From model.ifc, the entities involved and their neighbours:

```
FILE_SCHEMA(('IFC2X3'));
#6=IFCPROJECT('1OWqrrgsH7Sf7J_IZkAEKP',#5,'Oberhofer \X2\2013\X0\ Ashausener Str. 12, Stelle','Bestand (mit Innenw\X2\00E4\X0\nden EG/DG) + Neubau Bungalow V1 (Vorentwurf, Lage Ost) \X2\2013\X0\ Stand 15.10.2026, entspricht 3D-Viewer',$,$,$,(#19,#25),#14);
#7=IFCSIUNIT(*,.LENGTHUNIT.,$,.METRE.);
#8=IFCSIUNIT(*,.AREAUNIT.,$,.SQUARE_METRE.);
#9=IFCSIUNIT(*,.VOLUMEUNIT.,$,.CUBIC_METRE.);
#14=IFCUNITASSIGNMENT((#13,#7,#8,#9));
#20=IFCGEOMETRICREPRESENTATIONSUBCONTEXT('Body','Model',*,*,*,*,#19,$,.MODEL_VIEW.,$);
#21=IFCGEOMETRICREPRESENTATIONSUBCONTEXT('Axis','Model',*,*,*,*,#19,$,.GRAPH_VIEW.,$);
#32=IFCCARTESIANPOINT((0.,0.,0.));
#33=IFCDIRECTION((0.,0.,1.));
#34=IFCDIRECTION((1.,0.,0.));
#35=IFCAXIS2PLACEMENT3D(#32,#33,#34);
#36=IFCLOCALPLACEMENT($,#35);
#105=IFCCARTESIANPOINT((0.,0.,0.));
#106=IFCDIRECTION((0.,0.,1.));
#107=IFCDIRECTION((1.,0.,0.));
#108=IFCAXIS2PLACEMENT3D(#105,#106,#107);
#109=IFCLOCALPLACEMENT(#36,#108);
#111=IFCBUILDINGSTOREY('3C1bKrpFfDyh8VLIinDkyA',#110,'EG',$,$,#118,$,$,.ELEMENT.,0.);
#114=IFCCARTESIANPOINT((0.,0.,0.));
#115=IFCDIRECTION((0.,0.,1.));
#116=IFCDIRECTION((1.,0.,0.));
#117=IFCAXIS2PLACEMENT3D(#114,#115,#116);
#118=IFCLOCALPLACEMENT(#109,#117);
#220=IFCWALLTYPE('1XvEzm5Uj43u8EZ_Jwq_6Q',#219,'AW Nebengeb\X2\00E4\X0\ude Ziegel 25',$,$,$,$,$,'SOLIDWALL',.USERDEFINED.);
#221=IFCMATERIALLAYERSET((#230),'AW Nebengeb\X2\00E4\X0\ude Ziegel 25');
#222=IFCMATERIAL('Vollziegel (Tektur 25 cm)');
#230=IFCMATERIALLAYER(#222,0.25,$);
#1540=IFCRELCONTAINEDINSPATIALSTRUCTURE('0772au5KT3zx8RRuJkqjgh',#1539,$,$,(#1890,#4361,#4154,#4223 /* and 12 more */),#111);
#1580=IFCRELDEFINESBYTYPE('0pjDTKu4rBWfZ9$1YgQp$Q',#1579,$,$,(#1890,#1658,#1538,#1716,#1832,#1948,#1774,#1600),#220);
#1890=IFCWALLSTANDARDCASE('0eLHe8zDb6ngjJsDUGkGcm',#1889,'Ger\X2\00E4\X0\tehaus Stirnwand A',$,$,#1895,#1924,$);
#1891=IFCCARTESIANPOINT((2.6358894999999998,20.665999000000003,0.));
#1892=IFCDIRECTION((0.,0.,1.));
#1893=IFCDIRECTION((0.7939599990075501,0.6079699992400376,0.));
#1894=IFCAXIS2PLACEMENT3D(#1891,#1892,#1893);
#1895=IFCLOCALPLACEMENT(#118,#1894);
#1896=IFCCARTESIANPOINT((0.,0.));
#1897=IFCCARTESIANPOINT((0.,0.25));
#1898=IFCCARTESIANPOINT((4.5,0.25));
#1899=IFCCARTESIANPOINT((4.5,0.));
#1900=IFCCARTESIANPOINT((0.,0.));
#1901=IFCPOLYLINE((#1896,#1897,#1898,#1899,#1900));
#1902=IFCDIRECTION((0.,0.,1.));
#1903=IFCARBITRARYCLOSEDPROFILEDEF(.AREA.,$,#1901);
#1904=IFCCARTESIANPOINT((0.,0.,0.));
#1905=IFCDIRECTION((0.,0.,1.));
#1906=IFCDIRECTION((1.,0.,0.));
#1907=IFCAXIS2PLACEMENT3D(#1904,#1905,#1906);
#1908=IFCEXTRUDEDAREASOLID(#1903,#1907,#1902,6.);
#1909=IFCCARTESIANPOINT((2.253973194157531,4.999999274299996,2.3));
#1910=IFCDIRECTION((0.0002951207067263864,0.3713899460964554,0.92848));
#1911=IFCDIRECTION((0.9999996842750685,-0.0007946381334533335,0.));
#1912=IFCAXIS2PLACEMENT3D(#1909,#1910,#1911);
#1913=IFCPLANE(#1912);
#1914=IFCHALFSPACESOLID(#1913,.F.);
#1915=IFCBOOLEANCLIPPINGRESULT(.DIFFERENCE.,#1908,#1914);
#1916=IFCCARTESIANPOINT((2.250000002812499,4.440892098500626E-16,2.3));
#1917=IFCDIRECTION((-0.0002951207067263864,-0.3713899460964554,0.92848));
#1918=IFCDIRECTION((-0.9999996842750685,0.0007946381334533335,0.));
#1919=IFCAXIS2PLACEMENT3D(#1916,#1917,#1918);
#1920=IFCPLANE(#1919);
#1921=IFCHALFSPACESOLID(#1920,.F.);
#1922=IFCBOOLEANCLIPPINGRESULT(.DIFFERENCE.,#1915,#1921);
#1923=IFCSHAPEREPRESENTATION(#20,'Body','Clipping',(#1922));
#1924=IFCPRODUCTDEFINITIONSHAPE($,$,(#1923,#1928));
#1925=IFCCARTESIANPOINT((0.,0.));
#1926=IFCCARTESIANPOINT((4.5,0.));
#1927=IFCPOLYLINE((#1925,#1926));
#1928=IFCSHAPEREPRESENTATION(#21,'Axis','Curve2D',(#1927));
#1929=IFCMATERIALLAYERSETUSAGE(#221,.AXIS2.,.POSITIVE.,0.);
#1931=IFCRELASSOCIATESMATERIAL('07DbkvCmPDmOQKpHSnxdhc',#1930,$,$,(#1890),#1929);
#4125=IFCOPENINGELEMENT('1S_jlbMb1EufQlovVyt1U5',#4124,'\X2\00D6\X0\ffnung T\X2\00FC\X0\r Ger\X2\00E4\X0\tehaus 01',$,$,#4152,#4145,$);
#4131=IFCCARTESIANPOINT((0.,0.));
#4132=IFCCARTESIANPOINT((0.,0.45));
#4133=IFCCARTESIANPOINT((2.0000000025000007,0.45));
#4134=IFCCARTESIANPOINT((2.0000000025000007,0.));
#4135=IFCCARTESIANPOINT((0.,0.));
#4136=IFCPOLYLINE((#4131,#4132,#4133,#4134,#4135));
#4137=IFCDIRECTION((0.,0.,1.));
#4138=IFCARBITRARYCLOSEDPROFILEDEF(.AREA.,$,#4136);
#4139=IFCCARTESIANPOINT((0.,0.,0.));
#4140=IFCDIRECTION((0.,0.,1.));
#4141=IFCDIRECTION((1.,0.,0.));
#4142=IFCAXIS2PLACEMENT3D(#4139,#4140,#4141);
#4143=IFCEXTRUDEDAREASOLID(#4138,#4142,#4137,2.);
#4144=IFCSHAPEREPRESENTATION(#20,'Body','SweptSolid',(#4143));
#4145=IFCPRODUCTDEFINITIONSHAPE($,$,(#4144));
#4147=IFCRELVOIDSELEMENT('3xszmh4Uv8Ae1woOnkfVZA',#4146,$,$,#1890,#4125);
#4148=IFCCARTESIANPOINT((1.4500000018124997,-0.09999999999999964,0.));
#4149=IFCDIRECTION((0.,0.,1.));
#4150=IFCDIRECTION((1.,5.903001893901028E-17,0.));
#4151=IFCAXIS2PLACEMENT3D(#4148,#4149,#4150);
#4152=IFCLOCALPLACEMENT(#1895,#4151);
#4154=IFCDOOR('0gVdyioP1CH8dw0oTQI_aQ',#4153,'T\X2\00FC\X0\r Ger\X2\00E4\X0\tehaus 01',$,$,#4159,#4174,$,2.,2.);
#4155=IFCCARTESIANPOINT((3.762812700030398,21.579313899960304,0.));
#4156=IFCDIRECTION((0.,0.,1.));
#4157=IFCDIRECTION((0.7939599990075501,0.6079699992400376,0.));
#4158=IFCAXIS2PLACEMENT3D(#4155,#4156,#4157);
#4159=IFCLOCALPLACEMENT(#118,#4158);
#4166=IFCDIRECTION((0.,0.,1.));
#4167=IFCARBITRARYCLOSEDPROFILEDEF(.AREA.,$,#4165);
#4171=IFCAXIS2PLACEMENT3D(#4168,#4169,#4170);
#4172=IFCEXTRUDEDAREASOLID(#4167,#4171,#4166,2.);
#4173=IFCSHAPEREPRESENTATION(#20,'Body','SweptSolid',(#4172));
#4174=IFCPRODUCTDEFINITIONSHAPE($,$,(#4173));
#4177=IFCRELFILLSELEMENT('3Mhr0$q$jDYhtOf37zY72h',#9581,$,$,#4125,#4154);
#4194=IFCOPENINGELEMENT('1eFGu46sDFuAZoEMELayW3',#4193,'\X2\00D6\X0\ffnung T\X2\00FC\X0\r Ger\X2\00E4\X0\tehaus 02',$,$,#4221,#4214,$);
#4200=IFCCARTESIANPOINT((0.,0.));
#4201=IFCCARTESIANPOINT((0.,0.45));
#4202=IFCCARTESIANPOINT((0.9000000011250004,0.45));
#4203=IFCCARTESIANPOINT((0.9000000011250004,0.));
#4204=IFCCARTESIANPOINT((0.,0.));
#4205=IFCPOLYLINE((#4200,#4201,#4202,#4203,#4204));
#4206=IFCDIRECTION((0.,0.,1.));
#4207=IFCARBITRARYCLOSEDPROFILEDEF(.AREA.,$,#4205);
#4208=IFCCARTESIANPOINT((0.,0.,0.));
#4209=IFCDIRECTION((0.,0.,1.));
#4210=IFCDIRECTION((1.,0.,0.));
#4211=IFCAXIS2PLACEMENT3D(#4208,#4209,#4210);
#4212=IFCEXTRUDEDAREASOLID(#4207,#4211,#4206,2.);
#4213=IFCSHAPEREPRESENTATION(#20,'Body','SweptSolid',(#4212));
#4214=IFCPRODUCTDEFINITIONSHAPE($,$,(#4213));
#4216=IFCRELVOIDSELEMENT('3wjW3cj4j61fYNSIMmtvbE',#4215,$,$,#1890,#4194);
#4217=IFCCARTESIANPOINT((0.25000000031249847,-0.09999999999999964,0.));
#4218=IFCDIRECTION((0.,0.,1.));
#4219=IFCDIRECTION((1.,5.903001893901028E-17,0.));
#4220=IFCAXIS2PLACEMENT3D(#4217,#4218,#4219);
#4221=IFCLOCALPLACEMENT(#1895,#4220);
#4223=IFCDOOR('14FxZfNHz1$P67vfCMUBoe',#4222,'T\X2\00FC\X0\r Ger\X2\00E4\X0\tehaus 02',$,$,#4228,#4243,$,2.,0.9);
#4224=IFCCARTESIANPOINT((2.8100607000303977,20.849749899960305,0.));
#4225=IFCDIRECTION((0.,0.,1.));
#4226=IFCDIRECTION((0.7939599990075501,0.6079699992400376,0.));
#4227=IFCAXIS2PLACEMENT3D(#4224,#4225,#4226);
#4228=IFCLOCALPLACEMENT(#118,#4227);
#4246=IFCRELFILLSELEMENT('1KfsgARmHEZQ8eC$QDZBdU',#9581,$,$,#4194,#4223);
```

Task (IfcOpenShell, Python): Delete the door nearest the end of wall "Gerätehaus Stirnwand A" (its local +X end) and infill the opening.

```python
import ifcopenshell
import ifcopenshell.api.feature
import ifcopenshell.api.root
import ifcopenshell.geom
import ifcopenshell.util.shape

model = ifcopenshell.open("model.ifc")
settings = ifcopenshell.geom.settings()


def volume(element):
    """Net volume in cubic metres, openings subtracted."""
    shape = ifcopenshell.geom.create_shape(settings, element)
    return ifcopenshell.util.shape.get_volume(shape.geometry)


door = model.by_id(4154)
opening = door.FillsVoids[0].RelatingOpeningElement
wall = opening.VoidsElements[0].RelatingBuildingElement
before = volume(wall)

ifcopenshell.api.root.remove_product(model, product=door)
ifcopenshell.api.feature.remove_feature(model, feature=opening)

after = volume(wall)

print(f"wall volume {before:.3f} -> {after:.3f} m3")

model.write("model_updated.ifc")
```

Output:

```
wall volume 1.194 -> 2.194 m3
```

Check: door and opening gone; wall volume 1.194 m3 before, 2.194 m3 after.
